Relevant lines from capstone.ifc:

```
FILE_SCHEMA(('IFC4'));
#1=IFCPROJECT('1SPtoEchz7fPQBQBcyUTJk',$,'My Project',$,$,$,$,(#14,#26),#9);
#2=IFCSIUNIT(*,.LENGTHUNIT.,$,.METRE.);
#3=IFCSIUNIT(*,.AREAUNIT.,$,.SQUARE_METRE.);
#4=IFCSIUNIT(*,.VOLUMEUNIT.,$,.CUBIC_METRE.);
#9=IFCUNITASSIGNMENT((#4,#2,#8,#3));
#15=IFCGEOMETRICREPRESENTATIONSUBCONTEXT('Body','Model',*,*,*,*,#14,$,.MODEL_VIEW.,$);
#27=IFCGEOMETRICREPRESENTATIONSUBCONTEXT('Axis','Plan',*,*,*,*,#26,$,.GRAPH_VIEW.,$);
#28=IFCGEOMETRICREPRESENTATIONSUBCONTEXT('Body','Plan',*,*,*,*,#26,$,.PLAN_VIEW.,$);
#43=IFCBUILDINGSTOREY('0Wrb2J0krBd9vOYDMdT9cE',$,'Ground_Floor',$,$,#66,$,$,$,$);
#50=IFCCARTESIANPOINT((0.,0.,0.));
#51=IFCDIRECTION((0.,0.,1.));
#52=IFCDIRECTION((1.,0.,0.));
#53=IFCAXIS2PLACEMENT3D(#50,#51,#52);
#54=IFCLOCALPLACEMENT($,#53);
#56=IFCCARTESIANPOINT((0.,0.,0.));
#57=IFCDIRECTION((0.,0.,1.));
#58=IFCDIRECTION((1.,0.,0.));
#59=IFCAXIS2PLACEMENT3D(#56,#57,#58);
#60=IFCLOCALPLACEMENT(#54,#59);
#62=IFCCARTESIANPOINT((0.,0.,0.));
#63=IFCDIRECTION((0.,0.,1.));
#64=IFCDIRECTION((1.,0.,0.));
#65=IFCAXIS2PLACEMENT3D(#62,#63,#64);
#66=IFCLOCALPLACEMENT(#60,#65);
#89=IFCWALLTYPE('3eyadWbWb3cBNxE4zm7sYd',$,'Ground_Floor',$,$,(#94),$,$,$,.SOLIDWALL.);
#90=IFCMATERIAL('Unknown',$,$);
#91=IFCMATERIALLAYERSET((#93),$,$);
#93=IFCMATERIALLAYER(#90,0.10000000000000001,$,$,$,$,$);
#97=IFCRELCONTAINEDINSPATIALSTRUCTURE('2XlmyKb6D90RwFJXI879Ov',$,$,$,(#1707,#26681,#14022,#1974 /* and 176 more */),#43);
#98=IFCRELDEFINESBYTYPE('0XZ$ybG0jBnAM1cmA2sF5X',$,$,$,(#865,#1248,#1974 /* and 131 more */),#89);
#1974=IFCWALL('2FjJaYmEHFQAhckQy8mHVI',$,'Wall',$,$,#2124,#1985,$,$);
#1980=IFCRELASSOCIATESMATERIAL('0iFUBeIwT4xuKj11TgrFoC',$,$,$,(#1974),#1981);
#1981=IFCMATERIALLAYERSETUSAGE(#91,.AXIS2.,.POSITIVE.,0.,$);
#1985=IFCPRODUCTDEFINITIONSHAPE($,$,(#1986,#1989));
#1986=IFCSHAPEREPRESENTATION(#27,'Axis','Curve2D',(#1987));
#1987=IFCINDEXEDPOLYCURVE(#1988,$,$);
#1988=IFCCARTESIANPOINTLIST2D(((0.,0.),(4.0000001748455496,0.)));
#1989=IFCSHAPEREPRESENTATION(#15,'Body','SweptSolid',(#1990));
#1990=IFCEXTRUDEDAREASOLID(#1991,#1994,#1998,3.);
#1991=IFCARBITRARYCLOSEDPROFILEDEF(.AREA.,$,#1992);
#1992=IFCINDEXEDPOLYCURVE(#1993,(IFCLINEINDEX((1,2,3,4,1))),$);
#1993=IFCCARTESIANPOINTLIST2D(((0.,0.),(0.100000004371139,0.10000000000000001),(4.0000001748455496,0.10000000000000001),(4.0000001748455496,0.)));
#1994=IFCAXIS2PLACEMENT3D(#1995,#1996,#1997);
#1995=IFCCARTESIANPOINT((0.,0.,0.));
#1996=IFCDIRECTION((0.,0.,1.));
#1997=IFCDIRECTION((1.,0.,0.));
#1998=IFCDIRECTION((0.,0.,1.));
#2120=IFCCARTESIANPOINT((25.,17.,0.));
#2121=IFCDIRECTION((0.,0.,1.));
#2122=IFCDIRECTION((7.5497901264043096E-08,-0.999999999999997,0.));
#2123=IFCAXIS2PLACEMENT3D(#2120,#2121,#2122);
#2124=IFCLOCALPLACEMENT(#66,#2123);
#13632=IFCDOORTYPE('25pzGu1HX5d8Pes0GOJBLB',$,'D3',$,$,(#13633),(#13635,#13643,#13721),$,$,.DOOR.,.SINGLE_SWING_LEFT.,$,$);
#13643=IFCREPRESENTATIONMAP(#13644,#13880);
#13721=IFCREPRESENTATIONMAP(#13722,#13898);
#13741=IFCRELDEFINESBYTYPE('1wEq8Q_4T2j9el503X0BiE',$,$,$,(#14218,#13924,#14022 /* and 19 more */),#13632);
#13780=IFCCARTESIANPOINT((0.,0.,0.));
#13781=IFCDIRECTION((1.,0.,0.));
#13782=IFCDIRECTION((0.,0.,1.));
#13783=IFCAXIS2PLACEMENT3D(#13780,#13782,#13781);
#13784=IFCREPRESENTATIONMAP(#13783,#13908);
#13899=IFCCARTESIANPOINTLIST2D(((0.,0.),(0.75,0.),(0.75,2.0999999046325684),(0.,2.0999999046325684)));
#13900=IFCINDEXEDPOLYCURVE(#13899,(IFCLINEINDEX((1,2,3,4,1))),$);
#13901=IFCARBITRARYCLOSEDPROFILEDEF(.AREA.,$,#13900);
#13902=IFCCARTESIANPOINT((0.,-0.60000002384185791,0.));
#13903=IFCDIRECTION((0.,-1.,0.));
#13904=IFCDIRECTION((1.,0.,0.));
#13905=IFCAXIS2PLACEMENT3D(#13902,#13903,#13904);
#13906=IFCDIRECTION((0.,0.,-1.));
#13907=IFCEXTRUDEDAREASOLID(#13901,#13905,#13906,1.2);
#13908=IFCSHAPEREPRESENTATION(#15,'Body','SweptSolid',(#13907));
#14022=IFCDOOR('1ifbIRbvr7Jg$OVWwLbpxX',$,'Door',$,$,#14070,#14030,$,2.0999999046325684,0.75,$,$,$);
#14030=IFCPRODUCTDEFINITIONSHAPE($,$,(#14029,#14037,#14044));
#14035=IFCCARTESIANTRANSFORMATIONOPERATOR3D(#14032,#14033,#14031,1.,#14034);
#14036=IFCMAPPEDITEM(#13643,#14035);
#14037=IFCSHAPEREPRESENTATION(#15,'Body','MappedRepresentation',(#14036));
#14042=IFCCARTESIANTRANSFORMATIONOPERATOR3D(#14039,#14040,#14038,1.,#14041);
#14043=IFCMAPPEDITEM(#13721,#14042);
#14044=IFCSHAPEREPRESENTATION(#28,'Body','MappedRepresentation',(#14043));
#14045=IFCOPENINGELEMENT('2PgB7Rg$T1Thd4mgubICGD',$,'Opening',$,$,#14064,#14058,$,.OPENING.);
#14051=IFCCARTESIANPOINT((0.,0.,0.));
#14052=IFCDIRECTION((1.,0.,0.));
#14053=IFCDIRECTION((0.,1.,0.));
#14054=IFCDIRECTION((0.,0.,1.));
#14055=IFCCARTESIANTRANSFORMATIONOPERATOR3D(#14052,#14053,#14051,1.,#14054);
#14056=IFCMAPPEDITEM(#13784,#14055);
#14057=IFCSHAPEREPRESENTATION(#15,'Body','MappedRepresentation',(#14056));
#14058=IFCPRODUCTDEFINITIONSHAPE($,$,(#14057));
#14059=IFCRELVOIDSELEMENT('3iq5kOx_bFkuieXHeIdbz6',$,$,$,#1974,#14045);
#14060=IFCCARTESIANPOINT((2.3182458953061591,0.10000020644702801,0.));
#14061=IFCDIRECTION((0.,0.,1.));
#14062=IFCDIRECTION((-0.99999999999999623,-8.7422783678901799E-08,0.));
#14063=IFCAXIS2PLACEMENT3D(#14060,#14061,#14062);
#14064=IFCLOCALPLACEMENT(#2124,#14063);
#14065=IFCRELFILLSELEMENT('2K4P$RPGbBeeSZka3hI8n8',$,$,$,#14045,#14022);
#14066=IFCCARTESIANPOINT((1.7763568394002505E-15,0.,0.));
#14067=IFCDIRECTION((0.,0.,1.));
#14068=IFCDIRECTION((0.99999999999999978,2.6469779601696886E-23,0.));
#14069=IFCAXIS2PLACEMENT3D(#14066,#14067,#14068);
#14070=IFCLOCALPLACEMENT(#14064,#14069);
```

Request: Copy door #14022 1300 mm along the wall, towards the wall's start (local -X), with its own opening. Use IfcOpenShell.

```python
import ifcopenshell
import ifcopenshell.api.feature
import ifcopenshell.api.geometry
import ifcopenshell.api.root
import ifcopenshell.geom
import ifcopenshell.util.element
import ifcopenshell.util.placement
import ifcopenshell.util.shape
import ifcopenshell.util.unit

model = ifcopenshell.open("capstone.ifc")
unit_scale = ifcopenshell.util.unit.calculate_unit_scale(model)
settings = ifcopenshell.geom.settings()


def volume(element):
    """Net volume in cubic metres, openings subtracted."""
    shape = ifcopenshell.geom.create_shape(settings, element)
    return ifcopenshell.util.shape.get_volume(shape.geometry)


door = model.by_guid("1ifbIRbvr7Jg$OVWwLbpxX")
opening = door.FillsVoids[0].RelatingOpeningElement
wall = opening.VoidsElements[0].RelatingBuildingElement
before = volume(wall)
shift = ifcopenshell.util.placement.get_local_placement(wall.ObjectPlacement)[:3, 0] * -1.3 / unit_scale

# copy_class copies the void relationship, type, container and properties, but no geometry.
new_opening = ifcopenshell.api.root.copy_class(model, product=opening)
new_opening.Representation = ifcopenshell.util.element.copy_deep(
    model, opening.Representation, exclude=["IfcGeometricRepresentationContext", "IfcRepresentationMap"]
)
new_door = ifcopenshell.api.root.copy_class(model, product=door)
new_door.Representation = ifcopenshell.util.element.copy_deep(
    model, door.Representation, exclude=["IfcGeometricRepresentationContext", "IfcRepresentationMap"]
)
ifcopenshell.api.feature.add_filling(model, opening=new_opening, element=new_door)

for old, new in ((opening, new_opening), (door, new_door)):
    matrix = ifcopenshell.util.placement.get_local_placement(old.ObjectPlacement)
    matrix[:3, 3] += shift
    ifcopenshell.api.geometry.edit_object_placement(model, product=new, matrix=matrix, is_si=False)

after = volume(wall)

print(f"wall volume {before:.3f} -> {after:.3f} m3")

model.write("capstone-out.ifc")
```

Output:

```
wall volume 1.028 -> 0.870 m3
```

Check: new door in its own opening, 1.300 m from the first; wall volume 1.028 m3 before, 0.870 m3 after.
